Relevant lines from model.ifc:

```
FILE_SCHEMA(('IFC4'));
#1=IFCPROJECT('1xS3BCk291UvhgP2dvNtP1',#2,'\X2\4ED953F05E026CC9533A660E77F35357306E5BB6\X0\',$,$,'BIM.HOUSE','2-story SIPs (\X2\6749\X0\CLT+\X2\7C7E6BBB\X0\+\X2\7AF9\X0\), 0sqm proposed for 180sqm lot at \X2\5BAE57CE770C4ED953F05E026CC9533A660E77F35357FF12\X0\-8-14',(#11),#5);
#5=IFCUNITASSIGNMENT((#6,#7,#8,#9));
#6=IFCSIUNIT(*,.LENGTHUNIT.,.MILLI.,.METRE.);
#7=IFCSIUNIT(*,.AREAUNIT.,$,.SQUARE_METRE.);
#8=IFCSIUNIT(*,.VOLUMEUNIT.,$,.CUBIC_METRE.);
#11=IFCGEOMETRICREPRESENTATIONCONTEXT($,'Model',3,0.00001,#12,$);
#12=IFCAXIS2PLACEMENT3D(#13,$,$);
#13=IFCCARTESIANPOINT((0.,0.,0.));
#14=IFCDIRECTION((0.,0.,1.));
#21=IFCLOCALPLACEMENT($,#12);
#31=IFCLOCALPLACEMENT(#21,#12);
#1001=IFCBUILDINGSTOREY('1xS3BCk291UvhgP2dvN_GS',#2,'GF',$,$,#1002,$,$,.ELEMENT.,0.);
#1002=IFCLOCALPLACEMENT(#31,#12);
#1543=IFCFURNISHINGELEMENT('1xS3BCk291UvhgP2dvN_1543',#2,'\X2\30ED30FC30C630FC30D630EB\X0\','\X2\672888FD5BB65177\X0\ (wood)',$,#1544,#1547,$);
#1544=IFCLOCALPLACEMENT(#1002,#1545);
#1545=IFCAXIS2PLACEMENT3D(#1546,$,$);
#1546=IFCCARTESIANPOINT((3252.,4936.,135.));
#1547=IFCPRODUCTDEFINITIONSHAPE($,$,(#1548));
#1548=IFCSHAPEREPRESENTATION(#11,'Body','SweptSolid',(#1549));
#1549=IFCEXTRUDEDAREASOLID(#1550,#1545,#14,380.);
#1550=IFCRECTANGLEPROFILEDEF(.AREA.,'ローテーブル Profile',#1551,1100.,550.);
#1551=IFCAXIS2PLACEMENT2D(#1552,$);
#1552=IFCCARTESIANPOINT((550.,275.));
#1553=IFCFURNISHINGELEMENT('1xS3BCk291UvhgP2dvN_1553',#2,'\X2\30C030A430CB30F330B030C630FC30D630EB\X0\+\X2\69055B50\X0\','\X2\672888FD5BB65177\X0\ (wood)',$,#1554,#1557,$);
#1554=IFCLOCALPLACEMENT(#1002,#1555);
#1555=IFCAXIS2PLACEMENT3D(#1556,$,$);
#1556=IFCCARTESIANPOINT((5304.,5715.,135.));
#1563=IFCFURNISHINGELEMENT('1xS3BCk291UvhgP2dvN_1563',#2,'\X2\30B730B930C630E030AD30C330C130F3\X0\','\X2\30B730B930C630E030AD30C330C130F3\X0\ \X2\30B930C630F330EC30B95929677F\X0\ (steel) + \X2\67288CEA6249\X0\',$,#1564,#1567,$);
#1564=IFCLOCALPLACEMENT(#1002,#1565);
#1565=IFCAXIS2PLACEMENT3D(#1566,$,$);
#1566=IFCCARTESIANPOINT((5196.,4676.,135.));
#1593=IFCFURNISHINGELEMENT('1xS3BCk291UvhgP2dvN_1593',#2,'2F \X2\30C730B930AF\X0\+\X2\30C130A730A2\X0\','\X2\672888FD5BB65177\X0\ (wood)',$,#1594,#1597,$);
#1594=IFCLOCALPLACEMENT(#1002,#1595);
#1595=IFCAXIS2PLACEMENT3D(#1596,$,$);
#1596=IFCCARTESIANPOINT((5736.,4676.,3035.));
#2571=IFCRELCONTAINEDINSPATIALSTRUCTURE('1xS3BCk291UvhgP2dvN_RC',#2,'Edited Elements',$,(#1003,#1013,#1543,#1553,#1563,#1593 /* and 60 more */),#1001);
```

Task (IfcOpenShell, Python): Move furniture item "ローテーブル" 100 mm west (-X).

```python
import ifcopenshell
import ifcopenshell.api.geometry
import ifcopenshell.util.placement

model = ifcopenshell.open("model.ifc")

item = model.by_guid("1xS3BCk291UvhgP2dvN_1543")
matrix = ifcopenshell.util.placement.get_local_placement(item.ObjectPlacement)
matrix[0, 3] -= 100.0
ifcopenshell.api.geometry.edit_object_placement(model, product=item, matrix=matrix, is_si=False)

print(ifcopenshell.util.placement.get_local_placement(item.ObjectPlacement).round(3) + 0.0)

model.write("model_rev.ifc")
```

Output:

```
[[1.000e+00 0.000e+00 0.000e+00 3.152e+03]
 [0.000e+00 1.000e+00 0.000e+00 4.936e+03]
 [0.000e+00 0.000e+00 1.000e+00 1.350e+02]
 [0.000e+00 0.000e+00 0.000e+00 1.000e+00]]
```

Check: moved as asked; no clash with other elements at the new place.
